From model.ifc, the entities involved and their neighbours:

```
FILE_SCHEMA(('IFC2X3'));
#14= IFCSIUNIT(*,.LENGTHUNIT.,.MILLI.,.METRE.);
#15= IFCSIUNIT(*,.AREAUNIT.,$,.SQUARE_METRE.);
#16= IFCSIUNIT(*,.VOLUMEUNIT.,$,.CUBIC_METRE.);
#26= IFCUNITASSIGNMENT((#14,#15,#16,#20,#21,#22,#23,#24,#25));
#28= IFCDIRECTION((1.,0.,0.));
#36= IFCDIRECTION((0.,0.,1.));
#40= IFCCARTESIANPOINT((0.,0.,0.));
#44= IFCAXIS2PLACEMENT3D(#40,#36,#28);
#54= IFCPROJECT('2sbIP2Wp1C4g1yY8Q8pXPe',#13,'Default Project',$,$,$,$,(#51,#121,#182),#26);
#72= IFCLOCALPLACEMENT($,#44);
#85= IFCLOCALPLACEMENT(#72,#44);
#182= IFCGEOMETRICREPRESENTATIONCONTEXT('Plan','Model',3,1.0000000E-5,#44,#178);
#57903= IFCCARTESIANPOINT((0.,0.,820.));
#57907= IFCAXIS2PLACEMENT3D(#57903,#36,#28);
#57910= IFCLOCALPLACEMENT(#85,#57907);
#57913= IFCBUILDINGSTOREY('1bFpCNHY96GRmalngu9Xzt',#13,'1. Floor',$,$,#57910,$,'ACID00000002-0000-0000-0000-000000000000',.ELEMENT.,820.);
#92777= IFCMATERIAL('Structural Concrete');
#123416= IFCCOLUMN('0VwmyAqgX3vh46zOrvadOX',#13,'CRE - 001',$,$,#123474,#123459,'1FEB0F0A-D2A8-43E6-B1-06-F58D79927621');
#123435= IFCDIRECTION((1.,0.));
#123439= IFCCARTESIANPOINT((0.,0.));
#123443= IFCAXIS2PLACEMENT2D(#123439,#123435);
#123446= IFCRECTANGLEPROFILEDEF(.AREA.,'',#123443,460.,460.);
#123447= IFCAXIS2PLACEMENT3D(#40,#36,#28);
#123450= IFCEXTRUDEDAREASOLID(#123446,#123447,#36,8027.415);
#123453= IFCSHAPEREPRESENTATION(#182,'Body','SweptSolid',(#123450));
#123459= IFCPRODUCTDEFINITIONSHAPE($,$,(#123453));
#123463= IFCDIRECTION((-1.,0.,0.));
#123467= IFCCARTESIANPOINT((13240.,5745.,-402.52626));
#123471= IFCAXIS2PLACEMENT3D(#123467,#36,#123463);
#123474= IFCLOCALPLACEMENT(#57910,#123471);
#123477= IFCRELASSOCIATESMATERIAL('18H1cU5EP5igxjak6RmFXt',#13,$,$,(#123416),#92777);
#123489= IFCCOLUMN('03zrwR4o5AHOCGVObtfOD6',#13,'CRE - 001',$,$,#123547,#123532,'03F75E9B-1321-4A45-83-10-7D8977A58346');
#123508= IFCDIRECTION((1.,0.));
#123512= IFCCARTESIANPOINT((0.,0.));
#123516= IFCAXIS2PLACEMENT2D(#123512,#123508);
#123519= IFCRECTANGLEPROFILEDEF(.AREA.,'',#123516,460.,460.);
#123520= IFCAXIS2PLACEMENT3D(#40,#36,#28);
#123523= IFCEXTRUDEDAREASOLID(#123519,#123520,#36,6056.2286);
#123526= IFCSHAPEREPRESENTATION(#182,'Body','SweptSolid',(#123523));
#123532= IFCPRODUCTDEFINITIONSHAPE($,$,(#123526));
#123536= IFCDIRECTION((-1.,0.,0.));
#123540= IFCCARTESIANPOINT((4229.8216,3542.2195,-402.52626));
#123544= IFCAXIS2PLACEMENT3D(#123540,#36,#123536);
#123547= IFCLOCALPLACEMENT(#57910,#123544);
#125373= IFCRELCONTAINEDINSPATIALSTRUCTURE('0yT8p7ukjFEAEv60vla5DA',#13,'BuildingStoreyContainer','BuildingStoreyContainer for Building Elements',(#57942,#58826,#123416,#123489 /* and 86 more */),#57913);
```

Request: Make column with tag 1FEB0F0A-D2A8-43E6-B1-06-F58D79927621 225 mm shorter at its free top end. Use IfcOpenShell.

```python
import ifcopenshell
import ifcopenshell.util.unit

model = ifcopenshell.open("model.ifc")
unit_scale = ifcopenshell.util.unit.calculate_unit_scale(model)

member = model.by_guid("0VwmyAqgX3vh46zOrvadOX")
change = -0.225 / unit_scale

# The extrusion runs towards the end named, so only its depth changes.
body = next(r for r in member.Representation.Representations if r.RepresentationIdentifier == "Body")
solid = body.Items[0]
old_length = solid.Depth
solid.Depth += change

print(f"length {old_length:g} -> {solid.Depth:g}")

model.write("model_edited.ifc")
```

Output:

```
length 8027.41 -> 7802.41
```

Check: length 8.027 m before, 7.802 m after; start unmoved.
